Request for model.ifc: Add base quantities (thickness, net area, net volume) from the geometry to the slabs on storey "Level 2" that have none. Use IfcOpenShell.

First a look at what the model holds.

```python
import ifcopenshell
import ifcopenshell.util.element
import ifcopenshell.util.unit

model = ifcopenshell.open("model.ifc")
print(model.schema)
for unit_type in ("LENGTHUNIT", "AREAUNIT", "VOLUMEUNIT"):
    print(unit_type, ifcopenshell.util.unit.calculate_unit_scale(model, unit_type))
storey = next(s for s in model.by_type("IfcBuildingStorey") if s.Name == "Level 2")
slabs = [e for e in ifcopenshell.util.element.get_decomposition(storey) if e.is_a("IfcSlab")]
for e in sorted(slabs, key=lambda e: e.id()):
    print(e.id(), e.is_a(), e.Name, list(ifcopenshell.util.element.get_psets(e, qtos_only=True)), sep=" | ")
```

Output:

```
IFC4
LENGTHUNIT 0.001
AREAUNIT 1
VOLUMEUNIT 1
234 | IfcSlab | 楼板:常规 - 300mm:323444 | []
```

```python
import ifcopenshell
import ifcopenshell.api.pset
import ifcopenshell.geom
import ifcopenshell.util.element
import ifcopenshell.util.shape
import ifcopenshell.util.unit

model = ifcopenshell.open("model.ifc")
unit_scale = ifcopenshell.util.unit.calculate_unit_scale(model)
area_scale = ifcopenshell.util.unit.calculate_unit_scale(model, "AREAUNIT")
volume_scale = ifcopenshell.util.unit.calculate_unit_scale(model, "VOLUMEUNIT")
settings = ifcopenshell.geom.settings()

storey = next(s for s in model.by_type("IfcBuildingStorey") if s.Name == "Level 2")
slabs = [e for e in ifcopenshell.util.element.get_decomposition(storey) if e.is_a("IfcSlab")]

for e in sorted(slabs, key=lambda e: e.id()):
    if ifcopenshell.util.element.get_psets(e, qtos_only=True, should_inherit=False):
        continue
    # Geometry comes back in metres, in the element's own axes.
    shape = ifcopenshell.geom.create_shape(settings, e)
    values = {
        "Width": ifcopenshell.util.shape.get_z(shape.geometry) / unit_scale,
        "NetArea": ifcopenshell.util.shape.get_footprint_area(shape.geometry) / area_scale,
        "NetVolume": ifcopenshell.util.shape.get_volume(shape.geometry) / volume_scale,
    }
    qto = ifcopenshell.api.pset.add_qto(model, product=e, name="Qto_SlabBaseQuantities")
    ifcopenshell.api.pset.edit_qto(model, qto=qto, properties=values)
    print(e.id(), {k: round(v, 3) for k, v in values.items()})

model.write("model_v2.ifc")
```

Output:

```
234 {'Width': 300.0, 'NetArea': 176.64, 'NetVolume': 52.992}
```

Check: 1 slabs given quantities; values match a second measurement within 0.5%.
